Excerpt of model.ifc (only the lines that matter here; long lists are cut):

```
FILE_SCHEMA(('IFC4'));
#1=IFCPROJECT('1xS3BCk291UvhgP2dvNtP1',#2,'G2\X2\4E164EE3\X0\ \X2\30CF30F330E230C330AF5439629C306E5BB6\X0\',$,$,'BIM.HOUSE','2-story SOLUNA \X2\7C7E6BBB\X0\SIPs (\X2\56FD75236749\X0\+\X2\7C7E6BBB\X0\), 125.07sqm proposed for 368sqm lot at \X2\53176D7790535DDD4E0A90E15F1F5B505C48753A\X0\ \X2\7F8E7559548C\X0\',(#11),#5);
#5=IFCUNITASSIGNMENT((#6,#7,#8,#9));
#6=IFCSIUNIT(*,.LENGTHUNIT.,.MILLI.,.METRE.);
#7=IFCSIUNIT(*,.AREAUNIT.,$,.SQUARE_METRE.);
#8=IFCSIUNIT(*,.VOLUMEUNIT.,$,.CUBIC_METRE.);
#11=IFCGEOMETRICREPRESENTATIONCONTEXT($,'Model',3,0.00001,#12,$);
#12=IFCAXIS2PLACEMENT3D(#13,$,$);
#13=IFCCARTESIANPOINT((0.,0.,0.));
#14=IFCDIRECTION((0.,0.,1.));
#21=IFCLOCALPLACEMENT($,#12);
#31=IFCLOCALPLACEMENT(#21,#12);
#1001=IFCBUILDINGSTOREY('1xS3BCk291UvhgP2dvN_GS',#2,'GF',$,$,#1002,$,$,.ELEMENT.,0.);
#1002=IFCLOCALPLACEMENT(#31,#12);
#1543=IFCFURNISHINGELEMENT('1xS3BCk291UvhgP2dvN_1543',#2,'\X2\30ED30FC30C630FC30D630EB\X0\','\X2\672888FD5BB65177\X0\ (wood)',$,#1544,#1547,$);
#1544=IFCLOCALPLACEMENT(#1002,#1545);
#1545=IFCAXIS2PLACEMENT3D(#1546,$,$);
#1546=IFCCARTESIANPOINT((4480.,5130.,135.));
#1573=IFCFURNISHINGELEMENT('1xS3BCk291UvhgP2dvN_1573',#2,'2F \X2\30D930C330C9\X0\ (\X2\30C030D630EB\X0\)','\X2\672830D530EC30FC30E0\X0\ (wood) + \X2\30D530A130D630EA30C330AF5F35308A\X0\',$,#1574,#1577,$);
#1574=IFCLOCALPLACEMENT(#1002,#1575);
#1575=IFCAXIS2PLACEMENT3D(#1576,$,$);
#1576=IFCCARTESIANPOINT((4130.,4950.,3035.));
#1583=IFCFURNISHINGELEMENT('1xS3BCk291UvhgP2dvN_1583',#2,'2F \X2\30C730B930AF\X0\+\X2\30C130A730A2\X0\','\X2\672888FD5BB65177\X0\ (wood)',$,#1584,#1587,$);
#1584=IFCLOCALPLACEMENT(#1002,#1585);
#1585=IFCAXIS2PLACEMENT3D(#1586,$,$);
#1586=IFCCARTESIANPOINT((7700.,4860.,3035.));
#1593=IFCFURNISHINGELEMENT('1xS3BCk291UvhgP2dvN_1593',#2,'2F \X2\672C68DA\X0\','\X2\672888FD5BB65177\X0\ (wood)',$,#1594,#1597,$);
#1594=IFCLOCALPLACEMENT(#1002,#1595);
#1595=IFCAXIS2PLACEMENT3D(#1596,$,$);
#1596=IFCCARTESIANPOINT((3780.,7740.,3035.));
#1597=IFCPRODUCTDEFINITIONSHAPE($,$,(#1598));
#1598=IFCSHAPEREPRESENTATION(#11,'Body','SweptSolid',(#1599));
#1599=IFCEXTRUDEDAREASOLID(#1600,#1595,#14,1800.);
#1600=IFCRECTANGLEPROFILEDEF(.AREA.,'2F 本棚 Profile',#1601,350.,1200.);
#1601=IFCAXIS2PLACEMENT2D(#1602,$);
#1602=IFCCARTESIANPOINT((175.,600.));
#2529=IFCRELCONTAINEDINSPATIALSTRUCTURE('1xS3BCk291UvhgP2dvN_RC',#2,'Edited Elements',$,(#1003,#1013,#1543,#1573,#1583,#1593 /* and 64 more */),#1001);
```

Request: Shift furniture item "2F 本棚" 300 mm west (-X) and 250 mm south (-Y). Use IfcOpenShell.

```python
import ifcopenshell
import ifcopenshell.api.geometry
import ifcopenshell.util.placement
import ifcopenshell.util.unit

model = ifcopenshell.open("model.ifc")
unit_scale = ifcopenshell.util.unit.calculate_unit_scale(model)

item = model.by_guid("1xS3BCk291UvhgP2dvN_1593")
matrix = ifcopenshell.util.placement.get_local_placement(item.ObjectPlacement)
matrix[0, 3] -= 0.3 / unit_scale
matrix[1, 3] -= 0.25 / unit_scale
ifcopenshell.api.geometry.edit_object_placement(model, product=item, matrix=matrix, is_si=False)

print(ifcopenshell.util.placement.get_local_placement(item.ObjectPlacement).round(3) + 0.0)

model.write("model_rev.ifc")
```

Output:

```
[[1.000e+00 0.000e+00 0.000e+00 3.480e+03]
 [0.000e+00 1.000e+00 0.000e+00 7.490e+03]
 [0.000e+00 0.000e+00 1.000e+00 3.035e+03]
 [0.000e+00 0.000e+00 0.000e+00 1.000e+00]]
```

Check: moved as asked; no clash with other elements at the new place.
